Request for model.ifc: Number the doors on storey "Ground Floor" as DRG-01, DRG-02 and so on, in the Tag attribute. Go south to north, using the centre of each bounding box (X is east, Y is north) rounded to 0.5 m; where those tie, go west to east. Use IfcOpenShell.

First a look at what the model holds.

```python
import ifcopenshell
import ifcopenshell.util.element
import ifcopenshell.util.placement

model = ifcopenshell.open("model.ifc")
print(model.schema)
storey = next(s for s in model.by_type("IfcBuildingStorey") if s.Name == "Ground Floor")
doors = [e for e in ifcopenshell.util.element.get_decomposition(storey) if e.is_a("IfcDoor")]
for e in sorted(doors, key=lambda e: e.id()):
    origin = ifcopenshell.util.placement.get_local_placement(e.ObjectPlacement)[:3, 3]
    print(e.id(), e.Tag, e.Name, origin.round(2) + 0.0, sep=" | ")
```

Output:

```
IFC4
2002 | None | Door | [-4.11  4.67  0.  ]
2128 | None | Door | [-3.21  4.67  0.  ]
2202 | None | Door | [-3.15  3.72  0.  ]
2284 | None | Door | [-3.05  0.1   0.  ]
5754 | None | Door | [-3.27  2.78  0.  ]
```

```python
import ifcopenshell
import ifcopenshell.geom
import ifcopenshell.util.element
import ifcopenshell.util.shape

model = ifcopenshell.open("model.ifc")
settings = ifcopenshell.geom.settings()
settings.set("use-world-coords", True)


def centre(element):
    shape = ifcopenshell.geom.create_shape(settings, element)
    return ifcopenshell.util.shape.get_bbox_centroid(shape.geometry)


storey = next(s for s in model.by_type("IfcBuildingStorey") if s.Name == "Ground Floor")
doors = [e for e in ifcopenshell.util.element.get_decomposition(storey) if e.is_a("IfcDoor")]

# Insertion points can sit at a corner or the storey origin, so sort by the geometry (in metres).
centres = {e: centre(e) for e in doors}
doors.sort(key=lambda e: (round(centres[e][1] / 0.5), centres[e][0]))

for i, e in enumerate(doors, start=1):
    number = f"DRG-{i:02d}"
    e.Tag = number
    print(e.id(), number)

model.write("model-out.ifc")
```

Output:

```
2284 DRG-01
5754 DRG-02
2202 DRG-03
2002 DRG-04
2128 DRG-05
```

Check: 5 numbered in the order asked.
